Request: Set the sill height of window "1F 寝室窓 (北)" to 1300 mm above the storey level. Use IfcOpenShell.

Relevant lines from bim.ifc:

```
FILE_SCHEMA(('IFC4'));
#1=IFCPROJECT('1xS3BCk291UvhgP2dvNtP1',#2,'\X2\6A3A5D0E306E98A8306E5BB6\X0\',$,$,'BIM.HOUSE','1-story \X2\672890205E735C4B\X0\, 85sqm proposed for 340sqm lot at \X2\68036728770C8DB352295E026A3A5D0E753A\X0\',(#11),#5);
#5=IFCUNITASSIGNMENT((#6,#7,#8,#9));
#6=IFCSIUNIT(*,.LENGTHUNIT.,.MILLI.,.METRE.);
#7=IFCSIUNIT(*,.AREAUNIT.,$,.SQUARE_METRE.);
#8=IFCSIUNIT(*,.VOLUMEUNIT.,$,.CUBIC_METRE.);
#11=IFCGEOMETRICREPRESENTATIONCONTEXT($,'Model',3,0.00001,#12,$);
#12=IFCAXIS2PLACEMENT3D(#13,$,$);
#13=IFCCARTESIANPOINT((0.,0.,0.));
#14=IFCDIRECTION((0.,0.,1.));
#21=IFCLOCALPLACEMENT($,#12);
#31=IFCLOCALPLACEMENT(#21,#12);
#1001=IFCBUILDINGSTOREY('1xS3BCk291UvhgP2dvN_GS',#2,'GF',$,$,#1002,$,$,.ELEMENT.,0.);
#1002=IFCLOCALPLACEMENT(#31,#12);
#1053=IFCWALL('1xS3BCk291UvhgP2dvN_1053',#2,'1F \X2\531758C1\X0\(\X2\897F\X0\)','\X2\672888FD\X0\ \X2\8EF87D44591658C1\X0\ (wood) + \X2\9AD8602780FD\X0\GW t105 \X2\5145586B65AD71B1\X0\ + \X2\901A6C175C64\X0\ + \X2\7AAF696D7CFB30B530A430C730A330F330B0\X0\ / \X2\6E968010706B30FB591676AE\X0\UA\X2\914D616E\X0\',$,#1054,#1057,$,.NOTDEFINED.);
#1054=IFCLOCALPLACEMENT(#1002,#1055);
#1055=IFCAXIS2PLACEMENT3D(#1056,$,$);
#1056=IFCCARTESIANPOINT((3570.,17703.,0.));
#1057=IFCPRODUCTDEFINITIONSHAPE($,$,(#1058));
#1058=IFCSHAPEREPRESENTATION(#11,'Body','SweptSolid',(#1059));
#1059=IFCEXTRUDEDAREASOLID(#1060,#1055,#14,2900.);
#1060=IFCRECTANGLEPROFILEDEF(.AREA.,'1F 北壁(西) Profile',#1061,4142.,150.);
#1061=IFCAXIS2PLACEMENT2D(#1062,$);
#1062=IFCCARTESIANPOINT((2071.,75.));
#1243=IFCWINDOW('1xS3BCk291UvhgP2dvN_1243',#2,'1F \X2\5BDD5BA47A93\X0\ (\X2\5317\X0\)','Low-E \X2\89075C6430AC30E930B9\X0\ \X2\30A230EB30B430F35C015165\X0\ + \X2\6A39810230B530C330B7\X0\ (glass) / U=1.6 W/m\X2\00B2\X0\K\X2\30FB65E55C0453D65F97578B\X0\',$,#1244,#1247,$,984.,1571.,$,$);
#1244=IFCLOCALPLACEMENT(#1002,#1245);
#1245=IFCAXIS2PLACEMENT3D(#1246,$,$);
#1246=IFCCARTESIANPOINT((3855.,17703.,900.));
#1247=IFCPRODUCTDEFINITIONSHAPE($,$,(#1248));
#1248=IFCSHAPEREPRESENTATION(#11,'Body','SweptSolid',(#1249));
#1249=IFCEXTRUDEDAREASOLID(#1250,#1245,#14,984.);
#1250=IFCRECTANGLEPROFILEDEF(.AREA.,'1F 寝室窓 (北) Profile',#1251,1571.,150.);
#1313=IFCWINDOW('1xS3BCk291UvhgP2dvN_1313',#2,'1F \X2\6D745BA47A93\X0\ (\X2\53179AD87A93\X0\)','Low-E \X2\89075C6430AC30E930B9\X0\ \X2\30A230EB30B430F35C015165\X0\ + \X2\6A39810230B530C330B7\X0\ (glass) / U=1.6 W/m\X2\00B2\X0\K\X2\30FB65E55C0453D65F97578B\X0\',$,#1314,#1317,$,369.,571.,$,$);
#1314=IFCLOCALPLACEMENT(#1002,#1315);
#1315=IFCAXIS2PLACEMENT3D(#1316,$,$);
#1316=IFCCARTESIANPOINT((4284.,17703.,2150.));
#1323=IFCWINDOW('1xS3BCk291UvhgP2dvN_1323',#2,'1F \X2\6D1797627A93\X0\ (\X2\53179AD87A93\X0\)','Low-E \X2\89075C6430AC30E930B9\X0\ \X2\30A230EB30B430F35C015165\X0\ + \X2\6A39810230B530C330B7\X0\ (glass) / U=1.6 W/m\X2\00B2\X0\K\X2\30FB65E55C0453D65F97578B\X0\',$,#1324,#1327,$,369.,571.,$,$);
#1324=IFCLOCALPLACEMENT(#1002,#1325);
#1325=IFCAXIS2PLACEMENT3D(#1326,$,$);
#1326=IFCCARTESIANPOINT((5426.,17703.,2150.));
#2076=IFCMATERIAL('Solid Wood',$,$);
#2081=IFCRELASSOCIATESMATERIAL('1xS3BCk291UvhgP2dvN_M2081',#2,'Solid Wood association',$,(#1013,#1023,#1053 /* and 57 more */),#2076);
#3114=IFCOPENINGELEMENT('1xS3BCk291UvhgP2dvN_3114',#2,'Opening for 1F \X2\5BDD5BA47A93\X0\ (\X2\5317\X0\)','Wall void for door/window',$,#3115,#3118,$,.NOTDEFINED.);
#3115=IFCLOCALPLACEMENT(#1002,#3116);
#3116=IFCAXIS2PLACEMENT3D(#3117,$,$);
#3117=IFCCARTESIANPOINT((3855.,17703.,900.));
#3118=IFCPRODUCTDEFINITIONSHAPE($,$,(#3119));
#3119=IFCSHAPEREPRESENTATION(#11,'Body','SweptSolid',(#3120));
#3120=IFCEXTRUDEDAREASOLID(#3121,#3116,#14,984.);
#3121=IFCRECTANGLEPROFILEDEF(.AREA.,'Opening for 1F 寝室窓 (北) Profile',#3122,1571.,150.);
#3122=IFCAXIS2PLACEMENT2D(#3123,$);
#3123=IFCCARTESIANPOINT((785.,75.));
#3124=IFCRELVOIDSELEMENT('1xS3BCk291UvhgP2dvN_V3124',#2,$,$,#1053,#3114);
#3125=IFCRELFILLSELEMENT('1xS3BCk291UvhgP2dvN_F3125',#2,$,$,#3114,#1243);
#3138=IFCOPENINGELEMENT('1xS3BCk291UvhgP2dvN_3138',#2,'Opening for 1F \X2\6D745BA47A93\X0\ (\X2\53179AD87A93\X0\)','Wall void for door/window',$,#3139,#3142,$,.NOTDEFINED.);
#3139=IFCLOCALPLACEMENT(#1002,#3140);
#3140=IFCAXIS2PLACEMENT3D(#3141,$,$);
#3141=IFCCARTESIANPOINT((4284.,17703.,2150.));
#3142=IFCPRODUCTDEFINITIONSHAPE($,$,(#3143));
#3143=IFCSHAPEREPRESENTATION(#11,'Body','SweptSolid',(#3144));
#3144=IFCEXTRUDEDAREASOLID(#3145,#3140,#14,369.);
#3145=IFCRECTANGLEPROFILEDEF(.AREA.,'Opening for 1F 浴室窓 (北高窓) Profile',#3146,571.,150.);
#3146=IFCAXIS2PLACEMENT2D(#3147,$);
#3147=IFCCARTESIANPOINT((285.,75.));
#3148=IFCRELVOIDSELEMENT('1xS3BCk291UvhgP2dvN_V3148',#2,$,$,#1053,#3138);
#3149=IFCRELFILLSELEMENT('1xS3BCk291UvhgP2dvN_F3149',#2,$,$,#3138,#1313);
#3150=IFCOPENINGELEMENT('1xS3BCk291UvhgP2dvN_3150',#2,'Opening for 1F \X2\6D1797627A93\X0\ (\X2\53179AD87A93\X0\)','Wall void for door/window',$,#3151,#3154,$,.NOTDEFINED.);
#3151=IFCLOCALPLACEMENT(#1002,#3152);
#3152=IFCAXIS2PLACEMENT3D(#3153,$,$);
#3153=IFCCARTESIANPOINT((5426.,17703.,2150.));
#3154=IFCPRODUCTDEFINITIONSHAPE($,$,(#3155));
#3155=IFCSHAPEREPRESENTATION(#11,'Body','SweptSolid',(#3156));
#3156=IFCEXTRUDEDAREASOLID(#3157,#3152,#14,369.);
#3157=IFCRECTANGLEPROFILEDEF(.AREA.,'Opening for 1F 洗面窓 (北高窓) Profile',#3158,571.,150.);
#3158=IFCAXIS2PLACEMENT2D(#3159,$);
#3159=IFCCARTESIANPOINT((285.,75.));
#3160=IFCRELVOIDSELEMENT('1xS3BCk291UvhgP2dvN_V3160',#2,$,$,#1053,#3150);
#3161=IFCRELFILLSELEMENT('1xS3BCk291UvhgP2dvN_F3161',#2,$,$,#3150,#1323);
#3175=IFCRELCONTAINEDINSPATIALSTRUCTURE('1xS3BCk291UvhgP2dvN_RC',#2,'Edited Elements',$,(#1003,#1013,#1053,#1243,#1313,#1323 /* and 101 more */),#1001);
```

```python
import numpy as np
import ifcopenshell
import ifcopenshell.api.geometry
import ifcopenshell.geom
import ifcopenshell.util.element
import ifcopenshell.util.placement
import ifcopenshell.util.shape
import ifcopenshell.util.unit

model = ifcopenshell.open("bim.ifc")
unit_scale = ifcopenshell.util.unit.calculate_unit_scale(model)

window = model.by_id(1243)
opening = window.FillsVoids[0].RelatingOpeningElement
storey = ifcopenshell.util.element.get_container(window, ifc_class="IfcBuildingStorey")
level = ifcopenshell.util.placement.get_local_placement(storey.ObjectPlacement)[2, 3]

# The opening's origin need not be at the sill, so measure its lowest point.
shape = ifcopenshell.geom.create_shape(ifcopenshell.geom.settings(), opening)
bottom = ifcopenshell.util.shape.get_shape_bottom_elevation(shape, shape.geometry) / unit_scale
dz = level + 1300.0 - bottom

shift = np.array([0.0, 0.0, dz])
# The window is not placed relative to its opening, so move both.
for product in (opening, window):
    matrix = ifcopenshell.util.placement.get_local_placement(product.ObjectPlacement)
    matrix[:3, 3] += shift
    ifcopenshell.api.geometry.edit_object_placement(model, product=product, matrix=matrix, is_si=False)

print(f"moved by {dz * unit_scale:+.3f} m")

model.write("bim_rev.ifc")
```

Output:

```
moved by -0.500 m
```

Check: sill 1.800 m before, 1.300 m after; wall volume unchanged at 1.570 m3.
